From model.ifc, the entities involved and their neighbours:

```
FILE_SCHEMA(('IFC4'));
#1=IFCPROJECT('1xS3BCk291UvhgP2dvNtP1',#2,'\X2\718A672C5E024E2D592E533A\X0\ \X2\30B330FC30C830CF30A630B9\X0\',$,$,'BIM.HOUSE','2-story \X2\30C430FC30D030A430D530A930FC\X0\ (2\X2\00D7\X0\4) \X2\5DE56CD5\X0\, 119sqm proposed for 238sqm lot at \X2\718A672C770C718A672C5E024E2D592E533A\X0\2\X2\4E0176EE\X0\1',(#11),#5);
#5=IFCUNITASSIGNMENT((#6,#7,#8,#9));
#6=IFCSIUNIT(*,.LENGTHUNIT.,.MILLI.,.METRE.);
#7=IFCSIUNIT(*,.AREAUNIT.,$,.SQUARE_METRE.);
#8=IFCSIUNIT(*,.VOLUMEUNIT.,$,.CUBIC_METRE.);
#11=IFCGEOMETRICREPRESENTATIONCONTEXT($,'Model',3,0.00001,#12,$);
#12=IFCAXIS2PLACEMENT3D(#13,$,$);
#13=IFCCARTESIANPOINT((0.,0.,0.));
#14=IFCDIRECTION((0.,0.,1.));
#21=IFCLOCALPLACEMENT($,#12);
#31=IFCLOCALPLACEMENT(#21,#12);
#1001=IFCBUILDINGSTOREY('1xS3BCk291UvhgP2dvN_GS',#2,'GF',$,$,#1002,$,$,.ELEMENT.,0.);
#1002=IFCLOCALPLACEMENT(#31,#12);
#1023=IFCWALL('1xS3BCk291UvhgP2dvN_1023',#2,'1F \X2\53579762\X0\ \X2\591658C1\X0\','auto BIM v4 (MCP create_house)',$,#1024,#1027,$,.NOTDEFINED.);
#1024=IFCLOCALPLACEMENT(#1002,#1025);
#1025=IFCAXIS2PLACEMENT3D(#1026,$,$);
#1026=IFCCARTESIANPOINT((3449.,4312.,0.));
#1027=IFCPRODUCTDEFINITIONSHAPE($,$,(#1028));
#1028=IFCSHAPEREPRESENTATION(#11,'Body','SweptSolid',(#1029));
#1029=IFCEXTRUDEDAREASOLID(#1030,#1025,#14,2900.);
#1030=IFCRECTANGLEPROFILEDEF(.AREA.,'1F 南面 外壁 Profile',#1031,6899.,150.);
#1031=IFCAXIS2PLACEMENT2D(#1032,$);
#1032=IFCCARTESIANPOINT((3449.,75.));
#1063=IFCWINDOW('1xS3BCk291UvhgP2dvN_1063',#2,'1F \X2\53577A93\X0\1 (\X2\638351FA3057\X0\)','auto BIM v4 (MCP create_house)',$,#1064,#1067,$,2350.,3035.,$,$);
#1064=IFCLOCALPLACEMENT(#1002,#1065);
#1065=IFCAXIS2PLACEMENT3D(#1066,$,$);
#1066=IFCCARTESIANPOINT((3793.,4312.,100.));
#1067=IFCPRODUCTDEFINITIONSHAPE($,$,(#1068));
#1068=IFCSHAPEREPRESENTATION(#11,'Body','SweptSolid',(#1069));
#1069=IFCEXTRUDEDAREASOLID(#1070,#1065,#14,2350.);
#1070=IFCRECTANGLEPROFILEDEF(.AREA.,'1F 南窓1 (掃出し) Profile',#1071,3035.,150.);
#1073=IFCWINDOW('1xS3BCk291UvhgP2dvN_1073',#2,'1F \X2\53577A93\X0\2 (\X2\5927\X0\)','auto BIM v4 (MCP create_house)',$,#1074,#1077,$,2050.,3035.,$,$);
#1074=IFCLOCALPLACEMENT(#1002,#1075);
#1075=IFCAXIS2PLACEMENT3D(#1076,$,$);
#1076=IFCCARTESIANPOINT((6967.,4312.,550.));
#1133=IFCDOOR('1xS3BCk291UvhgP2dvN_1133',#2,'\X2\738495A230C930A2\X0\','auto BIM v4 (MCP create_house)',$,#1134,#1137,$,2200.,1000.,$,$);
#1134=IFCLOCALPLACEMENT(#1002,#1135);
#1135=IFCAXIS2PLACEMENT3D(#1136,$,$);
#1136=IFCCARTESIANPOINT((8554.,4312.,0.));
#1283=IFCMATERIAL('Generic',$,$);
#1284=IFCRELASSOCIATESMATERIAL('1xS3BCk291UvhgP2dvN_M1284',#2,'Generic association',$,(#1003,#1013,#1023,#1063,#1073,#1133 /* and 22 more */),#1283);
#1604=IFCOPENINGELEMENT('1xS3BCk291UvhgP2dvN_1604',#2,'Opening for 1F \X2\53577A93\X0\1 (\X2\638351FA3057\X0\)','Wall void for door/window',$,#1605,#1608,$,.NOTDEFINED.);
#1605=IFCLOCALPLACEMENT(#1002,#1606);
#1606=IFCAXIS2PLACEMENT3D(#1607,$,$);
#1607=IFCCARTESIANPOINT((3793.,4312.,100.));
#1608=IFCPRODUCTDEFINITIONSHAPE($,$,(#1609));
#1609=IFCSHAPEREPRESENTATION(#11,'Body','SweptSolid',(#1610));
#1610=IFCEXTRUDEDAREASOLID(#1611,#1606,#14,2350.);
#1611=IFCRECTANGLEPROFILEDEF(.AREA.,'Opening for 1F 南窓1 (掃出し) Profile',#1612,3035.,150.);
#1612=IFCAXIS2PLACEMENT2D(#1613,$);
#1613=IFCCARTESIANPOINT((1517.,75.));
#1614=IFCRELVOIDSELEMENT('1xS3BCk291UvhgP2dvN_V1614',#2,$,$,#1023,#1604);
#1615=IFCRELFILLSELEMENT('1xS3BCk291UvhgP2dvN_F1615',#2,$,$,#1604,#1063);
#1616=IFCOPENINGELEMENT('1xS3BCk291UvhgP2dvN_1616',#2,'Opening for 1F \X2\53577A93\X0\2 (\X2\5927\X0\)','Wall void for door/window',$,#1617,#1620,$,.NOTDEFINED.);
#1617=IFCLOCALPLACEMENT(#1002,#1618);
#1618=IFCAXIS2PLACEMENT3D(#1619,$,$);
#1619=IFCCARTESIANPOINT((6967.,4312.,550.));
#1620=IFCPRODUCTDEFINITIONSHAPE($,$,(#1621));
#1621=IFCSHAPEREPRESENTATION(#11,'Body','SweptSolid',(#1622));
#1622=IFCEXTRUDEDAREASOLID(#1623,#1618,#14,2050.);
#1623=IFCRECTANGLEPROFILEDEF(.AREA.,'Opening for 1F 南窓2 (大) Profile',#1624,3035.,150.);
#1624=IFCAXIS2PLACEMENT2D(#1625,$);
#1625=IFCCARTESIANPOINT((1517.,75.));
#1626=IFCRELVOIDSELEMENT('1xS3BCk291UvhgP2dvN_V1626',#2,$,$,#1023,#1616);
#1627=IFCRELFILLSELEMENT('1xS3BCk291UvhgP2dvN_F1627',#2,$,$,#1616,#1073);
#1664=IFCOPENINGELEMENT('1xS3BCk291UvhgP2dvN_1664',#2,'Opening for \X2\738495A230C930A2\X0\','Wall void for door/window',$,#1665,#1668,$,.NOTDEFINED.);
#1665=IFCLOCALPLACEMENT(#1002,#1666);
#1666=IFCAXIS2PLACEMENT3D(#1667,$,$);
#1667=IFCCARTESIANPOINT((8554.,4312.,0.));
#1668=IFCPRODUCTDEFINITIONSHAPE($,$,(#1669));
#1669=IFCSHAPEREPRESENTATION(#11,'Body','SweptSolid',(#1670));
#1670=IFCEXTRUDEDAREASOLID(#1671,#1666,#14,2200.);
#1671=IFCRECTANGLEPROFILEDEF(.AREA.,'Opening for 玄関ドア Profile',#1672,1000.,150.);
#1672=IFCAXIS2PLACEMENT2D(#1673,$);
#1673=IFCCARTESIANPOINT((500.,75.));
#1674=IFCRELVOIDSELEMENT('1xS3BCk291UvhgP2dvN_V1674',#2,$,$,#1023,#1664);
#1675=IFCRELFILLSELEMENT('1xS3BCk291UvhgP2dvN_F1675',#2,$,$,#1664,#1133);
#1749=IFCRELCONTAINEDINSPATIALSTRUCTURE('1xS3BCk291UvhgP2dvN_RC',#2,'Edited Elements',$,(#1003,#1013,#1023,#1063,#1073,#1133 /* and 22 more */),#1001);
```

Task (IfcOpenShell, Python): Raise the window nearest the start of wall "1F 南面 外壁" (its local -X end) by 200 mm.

```python
import numpy as np
import ifcopenshell
import ifcopenshell.api.geometry
import ifcopenshell.util.placement
import ifcopenshell.util.unit

model = ifcopenshell.open("model.ifc")
unit_scale = ifcopenshell.util.unit.calculate_unit_scale(model)

window = model.by_id(1063)
opening = window.FillsVoids[0].RelatingOpeningElement
dz = 0.2 / unit_scale

shift = np.array([0.0, 0.0, dz])
# The window is not placed relative to its opening, so move both.
for product in (opening, window):
    matrix = ifcopenshell.util.placement.get_local_placement(product.ObjectPlacement)
    matrix[:3, 3] += shift
    ifcopenshell.api.geometry.edit_object_placement(model, product=product, matrix=matrix, is_si=False)

print(f"moved by {dz * unit_scale:+.3f} m")

model.write("model_v2.ifc")
```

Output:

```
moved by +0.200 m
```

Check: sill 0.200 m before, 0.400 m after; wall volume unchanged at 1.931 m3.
